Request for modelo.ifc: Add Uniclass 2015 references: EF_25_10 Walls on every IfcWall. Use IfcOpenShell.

First a look at what the model holds.

```python
import ifcopenshell

model = ifcopenshell.open("modelo.ifc")
print(model.schema)
print("classifications:", [c.Name for c in model.by_type("IfcClassification")])
for ifc_class in ("IfcDoor", "IfcRoof", "IfcStair", "IfcWall", "IfcWindow"):
    print(ifc_class, len(model.by_type(ifc_class)))
```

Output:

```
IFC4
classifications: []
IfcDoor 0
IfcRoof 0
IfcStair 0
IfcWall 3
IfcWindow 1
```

```python
import ifcopenshell
import ifcopenshell.api.classification

model = ifcopenshell.open("modelo.ifc")

system = ifcopenshell.api.classification.add_classification(model, classification="Uniclass 2015")

codes = {
    "IfcWall": ("EF_25_10", "Walls"),
}
for ifc_class, (code, name) in codes.items():
    products = model.by_type(ifc_class)
    ifcopenshell.api.classification.add_reference(
        model, products=products, classification=system, identification=code, name=name
    )
    print(code, len(products))

model.write("modelo-out.ifc")
```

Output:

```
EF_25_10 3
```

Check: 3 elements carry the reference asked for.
